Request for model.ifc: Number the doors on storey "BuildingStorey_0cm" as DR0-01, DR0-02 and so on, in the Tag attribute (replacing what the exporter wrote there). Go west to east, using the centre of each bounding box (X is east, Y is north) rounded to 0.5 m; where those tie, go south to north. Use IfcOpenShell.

First a look at what the model holds.

```python
import ifcopenshell
import ifcopenshell.util.element
import ifcopenshell.util.placement

model = ifcopenshell.open("model.ifc")
print(model.schema)
storey = next(s for s in model.by_type("IfcBuildingStorey") if s.Name == "BuildingStorey_0cm")
doors = [e for e in ifcopenshell.util.element.get_decomposition(storey) if e.is_a("IfcDoor")]
for e in sorted(doors, key=lambda e: e.id()):
    origin = ifcopenshell.util.placement.get_local_placement(e.ObjectPlacement)[:3, 3]
    print(e.id(), e.Tag, e.Name, origin.round(2) + 0.0, sep=" | ")
```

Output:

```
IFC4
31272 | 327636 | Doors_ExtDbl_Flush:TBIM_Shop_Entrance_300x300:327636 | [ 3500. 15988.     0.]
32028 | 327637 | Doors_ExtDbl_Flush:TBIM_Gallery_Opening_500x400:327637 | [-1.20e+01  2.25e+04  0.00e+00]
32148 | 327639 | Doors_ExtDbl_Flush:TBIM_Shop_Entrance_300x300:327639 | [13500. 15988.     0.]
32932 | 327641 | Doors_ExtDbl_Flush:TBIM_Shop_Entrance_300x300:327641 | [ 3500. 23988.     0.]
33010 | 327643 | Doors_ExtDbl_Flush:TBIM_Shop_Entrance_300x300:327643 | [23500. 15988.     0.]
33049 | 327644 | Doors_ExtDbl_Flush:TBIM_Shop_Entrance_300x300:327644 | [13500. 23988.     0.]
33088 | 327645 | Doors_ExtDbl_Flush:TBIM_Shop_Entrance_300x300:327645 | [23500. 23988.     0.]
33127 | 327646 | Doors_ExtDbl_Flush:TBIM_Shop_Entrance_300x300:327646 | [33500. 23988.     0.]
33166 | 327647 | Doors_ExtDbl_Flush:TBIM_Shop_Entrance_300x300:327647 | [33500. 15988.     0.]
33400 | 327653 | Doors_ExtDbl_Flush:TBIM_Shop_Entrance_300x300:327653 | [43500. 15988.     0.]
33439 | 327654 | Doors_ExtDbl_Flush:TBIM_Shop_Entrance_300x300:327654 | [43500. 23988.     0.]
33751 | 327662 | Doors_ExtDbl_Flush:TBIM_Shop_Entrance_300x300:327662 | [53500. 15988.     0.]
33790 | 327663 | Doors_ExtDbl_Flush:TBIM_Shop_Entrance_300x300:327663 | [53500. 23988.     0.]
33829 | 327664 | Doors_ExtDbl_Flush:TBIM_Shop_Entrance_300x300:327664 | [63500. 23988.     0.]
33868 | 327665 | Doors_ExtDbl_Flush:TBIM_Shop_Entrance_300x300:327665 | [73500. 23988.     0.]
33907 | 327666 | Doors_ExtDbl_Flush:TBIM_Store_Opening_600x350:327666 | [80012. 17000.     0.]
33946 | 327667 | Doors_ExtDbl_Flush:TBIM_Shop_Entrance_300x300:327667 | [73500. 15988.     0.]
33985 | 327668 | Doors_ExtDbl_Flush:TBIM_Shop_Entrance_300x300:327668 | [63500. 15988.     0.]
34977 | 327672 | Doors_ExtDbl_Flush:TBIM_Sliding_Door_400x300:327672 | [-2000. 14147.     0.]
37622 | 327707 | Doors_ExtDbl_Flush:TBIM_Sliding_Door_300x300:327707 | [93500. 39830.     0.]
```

```python
import ifcopenshell
import ifcopenshell.geom
import ifcopenshell.util.element
import ifcopenshell.util.shape

model = ifcopenshell.open("model.ifc")
settings = ifcopenshell.geom.settings()
settings.set("use-world-coords", True)


def centre(element):
    shape = ifcopenshell.geom.create_shape(settings, element)
    return ifcopenshell.util.shape.get_bbox_centroid(shape.geometry)


storey = next(s for s in model.by_type("IfcBuildingStorey") if s.Name == "BuildingStorey_0cm")
doors = [e for e in ifcopenshell.util.element.get_decomposition(storey) if e.is_a("IfcDoor")]

# Insertion points can sit at a corner or the storey origin, so sort by the geometry (in metres).
centres = {e: centre(e) for e in doors}
doors.sort(key=lambda e: (round(centres[e][0] / 0.5), centres[e][1]))

for i, e in enumerate(doors, start=1):
    number = f"DR0-{i:02d}"
    e.Tag = number
    print(e.id(), number)

model.write("model_edited.ifc")
```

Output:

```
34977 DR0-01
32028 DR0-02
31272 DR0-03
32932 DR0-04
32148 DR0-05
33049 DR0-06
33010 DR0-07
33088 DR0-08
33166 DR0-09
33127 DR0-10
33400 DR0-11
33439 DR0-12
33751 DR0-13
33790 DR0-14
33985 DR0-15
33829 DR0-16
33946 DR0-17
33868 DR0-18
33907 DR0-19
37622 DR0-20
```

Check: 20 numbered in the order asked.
